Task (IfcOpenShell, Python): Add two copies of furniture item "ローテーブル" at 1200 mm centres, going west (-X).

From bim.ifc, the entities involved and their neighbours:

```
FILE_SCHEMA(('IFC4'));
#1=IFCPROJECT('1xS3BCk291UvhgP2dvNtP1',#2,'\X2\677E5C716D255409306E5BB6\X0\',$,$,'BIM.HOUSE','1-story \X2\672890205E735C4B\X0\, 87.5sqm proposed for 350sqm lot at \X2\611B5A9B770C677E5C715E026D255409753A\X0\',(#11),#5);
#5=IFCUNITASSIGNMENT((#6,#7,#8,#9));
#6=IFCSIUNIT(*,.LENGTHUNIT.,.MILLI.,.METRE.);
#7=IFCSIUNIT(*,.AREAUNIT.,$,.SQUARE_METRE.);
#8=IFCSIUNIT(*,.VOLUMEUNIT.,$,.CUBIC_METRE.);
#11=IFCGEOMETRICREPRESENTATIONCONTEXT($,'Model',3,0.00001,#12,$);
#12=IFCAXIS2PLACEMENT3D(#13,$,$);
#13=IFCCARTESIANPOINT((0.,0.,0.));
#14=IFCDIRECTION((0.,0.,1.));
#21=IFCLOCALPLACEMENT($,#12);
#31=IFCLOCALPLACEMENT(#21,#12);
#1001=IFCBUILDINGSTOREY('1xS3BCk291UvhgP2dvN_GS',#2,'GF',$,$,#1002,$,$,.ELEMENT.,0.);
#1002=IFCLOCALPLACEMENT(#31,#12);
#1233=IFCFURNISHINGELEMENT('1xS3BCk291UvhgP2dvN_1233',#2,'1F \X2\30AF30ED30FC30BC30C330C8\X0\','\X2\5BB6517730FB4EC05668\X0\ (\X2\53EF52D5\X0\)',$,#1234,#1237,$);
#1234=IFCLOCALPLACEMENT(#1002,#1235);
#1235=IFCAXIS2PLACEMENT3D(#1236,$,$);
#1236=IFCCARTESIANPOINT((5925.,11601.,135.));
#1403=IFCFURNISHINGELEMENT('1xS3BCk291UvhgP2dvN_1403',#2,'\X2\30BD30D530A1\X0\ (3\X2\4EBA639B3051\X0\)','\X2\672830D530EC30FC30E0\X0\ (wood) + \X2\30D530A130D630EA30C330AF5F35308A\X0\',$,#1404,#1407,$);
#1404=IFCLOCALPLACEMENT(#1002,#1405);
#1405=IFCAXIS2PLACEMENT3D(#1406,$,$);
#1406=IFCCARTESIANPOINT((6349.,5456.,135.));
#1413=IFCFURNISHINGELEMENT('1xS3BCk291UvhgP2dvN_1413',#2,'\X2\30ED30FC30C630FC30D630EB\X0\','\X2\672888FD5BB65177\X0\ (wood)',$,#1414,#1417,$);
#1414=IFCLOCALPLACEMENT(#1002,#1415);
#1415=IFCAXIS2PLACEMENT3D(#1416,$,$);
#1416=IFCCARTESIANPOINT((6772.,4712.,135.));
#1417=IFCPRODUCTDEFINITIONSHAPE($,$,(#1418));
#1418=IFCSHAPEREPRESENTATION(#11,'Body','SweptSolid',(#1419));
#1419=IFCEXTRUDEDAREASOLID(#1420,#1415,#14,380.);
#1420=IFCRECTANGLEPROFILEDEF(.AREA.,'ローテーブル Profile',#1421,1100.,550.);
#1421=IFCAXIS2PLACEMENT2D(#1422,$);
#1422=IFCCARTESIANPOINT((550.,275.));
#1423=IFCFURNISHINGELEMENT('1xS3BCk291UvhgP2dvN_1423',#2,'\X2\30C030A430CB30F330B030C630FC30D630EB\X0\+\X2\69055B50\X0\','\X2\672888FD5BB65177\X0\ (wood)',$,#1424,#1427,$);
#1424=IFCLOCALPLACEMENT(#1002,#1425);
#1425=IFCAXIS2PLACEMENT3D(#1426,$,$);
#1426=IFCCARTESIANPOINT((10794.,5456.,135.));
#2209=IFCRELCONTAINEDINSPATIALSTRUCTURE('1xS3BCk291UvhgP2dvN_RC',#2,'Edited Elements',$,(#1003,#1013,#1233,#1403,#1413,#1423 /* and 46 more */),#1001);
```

```python
import numpy as np
import ifcopenshell
import ifcopenshell.api.geometry
import ifcopenshell.api.root
import ifcopenshell.util.element
import ifcopenshell.util.placement

model = ifcopenshell.open("bim.ifc")


def reuse_history(source, copy):
    """copy_class also copies each property set's owner history, people and application; keep the originals."""
    for rel in copy.IsDefinedBy:
        if rel.is_a("IfcRelDefinesByProperties") and (history := rel.RelatingPropertyDefinition.OwnerHistory):
            rel.RelatingPropertyDefinition.OwnerHistory = source.OwnerHistory
            ifcopenshell.util.element.remove_deep2(model, history)


source = model.by_guid("1xS3BCk291UvhgP2dvN_1413")
base = ifcopenshell.util.placement.get_local_placement(source.ObjectPlacement)
step = np.array([-1.0, 0.0, 0.0]) * 1200.0

for i in range(1, 3):
    copy = ifcopenshell.api.root.copy_class(model, product=source)
    copy.Representation = ifcopenshell.util.element.copy_deep(
        model, source.Representation, exclude=["IfcGeometricRepresentationContext", "IfcRepresentationMap"]
    )
    reuse_history(source, copy)
    matrix = base.copy()
    matrix[:3, 3] += i * step
    print("added at", matrix[:3, 3].round(3) + 0.0)
    ifcopenshell.api.geometry.edit_object_placement(model, product=copy, matrix=matrix, is_si=False)

model.write("bim-out.ifc")
```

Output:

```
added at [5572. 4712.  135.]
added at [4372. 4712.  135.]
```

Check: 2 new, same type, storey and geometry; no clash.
